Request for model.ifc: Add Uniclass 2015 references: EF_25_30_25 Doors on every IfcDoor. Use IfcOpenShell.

First a look at what the model holds.

```python
import ifcopenshell

model = ifcopenshell.open("model.ifc")
print(model.schema)
print("classifications:", [c.Name for c in model.by_type("IfcClassification")])
for ifc_class in ("IfcDoor", "IfcRoof", "IfcStair", "IfcWall", "IfcWindow"):
    print(ifc_class, len(model.by_type(ifc_class)))
```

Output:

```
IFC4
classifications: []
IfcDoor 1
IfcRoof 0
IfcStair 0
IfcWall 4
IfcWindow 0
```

```python
import ifcopenshell
import ifcopenshell.api.classification

model = ifcopenshell.open("model.ifc")

system = ifcopenshell.api.classification.add_classification(model, classification="Uniclass 2015")

codes = {
    "IfcDoor": ("EF_25_30_25", "Doors"),
}
for ifc_class, (code, name) in codes.items():
    products = model.by_type(ifc_class)
    ifcopenshell.api.classification.add_reference(
        model, products=products, classification=system, identification=code, name=name
    )
    print(code, len(products))

model.write("model_rev.ifc")
```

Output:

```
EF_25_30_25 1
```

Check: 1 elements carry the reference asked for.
